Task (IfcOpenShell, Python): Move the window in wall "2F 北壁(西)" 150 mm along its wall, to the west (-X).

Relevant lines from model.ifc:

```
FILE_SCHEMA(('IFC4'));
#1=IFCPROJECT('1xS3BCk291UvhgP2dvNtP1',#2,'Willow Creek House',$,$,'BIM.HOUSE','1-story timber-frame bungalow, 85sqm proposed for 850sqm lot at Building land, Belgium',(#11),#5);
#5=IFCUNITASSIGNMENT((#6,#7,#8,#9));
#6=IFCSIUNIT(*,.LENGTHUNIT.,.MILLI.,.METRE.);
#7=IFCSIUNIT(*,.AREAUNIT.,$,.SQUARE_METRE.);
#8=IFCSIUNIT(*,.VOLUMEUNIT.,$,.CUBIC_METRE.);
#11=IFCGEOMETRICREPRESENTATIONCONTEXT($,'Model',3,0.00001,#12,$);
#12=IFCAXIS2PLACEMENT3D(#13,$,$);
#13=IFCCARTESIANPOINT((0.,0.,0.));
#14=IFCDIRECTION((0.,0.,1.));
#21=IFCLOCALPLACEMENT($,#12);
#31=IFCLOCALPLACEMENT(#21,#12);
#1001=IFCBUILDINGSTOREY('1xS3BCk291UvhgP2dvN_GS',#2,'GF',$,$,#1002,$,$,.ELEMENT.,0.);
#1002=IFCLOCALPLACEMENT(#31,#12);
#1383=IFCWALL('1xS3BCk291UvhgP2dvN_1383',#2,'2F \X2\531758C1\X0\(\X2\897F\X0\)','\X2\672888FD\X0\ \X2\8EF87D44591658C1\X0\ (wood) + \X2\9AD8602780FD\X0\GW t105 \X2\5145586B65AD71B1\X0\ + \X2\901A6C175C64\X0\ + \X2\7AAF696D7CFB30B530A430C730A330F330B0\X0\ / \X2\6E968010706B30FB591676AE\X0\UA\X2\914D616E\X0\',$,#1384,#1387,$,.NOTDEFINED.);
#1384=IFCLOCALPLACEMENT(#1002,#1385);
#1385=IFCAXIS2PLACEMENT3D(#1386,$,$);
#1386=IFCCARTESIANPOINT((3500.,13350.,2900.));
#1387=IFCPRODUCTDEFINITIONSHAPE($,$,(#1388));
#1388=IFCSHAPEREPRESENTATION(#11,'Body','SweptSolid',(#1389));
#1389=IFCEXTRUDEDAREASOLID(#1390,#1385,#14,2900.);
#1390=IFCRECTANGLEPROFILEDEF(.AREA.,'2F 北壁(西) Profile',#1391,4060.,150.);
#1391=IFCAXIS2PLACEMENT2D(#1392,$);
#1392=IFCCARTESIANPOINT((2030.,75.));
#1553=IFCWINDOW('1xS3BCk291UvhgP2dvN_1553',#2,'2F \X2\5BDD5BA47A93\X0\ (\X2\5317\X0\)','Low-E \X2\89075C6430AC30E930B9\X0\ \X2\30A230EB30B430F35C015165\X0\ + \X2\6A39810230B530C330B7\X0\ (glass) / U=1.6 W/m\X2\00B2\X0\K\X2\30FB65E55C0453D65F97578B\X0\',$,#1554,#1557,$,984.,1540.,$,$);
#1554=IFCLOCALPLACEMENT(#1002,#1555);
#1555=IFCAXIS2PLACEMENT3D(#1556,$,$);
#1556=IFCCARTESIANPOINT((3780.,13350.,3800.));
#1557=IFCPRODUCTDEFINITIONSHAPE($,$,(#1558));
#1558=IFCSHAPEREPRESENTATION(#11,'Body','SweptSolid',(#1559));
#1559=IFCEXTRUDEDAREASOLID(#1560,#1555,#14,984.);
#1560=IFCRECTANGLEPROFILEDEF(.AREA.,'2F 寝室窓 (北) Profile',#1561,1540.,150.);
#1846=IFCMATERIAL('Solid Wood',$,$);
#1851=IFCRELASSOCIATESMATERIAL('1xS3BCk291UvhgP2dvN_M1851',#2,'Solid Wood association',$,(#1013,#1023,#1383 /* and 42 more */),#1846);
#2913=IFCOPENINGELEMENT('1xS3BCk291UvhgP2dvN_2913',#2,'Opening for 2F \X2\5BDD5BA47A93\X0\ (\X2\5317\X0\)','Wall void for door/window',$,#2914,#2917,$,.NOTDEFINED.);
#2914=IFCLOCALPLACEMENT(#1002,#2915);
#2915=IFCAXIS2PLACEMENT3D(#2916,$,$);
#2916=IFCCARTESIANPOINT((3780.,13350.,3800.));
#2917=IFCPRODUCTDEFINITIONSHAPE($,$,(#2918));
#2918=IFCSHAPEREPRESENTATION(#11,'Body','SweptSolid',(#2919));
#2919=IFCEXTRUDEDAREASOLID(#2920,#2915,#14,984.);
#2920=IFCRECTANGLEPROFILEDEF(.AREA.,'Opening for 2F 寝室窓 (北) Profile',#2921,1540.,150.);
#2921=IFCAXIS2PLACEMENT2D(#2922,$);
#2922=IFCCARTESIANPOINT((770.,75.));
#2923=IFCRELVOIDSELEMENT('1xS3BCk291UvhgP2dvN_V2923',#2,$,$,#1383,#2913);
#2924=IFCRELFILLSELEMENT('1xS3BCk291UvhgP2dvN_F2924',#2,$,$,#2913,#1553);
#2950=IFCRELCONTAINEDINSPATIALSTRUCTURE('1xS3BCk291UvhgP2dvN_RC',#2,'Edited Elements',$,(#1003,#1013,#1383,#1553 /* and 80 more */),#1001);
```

```python
import ifcopenshell
import ifcopenshell.api.geometry
import ifcopenshell.util.placement
import ifcopenshell.util.unit

model = ifcopenshell.open("model.ifc")
unit_scale = ifcopenshell.util.unit.calculate_unit_scale(model)

window = model.by_guid("1xS3BCk291UvhgP2dvN_1553")
opening = window.FillsVoids[0].RelatingOpeningElement
wall = opening.VoidsElements[0].RelatingBuildingElement

wall_matrix = ifcopenshell.util.placement.get_local_placement(wall.ObjectPlacement)
shift = wall_matrix[:3, 0] * -0.15 / unit_scale
before = ifcopenshell.util.placement.get_local_placement(window.ObjectPlacement)[:3, 3].copy()

# The window is not placed relative to its opening, so move both.
for product in (opening, window):
    matrix = ifcopenshell.util.placement.get_local_placement(product.ObjectPlacement)
    matrix[:3, 3] += shift
    ifcopenshell.api.geometry.edit_object_placement(model, product=product, matrix=matrix, is_si=False)

after = ifcopenshell.util.placement.get_local_placement(window.ObjectPlacement)[:3, 3]
print("window moved by", (after - before).round(3) + 0.0)

model.write("model_v2.ifc")
```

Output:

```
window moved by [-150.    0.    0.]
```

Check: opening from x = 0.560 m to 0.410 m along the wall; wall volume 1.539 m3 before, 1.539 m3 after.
